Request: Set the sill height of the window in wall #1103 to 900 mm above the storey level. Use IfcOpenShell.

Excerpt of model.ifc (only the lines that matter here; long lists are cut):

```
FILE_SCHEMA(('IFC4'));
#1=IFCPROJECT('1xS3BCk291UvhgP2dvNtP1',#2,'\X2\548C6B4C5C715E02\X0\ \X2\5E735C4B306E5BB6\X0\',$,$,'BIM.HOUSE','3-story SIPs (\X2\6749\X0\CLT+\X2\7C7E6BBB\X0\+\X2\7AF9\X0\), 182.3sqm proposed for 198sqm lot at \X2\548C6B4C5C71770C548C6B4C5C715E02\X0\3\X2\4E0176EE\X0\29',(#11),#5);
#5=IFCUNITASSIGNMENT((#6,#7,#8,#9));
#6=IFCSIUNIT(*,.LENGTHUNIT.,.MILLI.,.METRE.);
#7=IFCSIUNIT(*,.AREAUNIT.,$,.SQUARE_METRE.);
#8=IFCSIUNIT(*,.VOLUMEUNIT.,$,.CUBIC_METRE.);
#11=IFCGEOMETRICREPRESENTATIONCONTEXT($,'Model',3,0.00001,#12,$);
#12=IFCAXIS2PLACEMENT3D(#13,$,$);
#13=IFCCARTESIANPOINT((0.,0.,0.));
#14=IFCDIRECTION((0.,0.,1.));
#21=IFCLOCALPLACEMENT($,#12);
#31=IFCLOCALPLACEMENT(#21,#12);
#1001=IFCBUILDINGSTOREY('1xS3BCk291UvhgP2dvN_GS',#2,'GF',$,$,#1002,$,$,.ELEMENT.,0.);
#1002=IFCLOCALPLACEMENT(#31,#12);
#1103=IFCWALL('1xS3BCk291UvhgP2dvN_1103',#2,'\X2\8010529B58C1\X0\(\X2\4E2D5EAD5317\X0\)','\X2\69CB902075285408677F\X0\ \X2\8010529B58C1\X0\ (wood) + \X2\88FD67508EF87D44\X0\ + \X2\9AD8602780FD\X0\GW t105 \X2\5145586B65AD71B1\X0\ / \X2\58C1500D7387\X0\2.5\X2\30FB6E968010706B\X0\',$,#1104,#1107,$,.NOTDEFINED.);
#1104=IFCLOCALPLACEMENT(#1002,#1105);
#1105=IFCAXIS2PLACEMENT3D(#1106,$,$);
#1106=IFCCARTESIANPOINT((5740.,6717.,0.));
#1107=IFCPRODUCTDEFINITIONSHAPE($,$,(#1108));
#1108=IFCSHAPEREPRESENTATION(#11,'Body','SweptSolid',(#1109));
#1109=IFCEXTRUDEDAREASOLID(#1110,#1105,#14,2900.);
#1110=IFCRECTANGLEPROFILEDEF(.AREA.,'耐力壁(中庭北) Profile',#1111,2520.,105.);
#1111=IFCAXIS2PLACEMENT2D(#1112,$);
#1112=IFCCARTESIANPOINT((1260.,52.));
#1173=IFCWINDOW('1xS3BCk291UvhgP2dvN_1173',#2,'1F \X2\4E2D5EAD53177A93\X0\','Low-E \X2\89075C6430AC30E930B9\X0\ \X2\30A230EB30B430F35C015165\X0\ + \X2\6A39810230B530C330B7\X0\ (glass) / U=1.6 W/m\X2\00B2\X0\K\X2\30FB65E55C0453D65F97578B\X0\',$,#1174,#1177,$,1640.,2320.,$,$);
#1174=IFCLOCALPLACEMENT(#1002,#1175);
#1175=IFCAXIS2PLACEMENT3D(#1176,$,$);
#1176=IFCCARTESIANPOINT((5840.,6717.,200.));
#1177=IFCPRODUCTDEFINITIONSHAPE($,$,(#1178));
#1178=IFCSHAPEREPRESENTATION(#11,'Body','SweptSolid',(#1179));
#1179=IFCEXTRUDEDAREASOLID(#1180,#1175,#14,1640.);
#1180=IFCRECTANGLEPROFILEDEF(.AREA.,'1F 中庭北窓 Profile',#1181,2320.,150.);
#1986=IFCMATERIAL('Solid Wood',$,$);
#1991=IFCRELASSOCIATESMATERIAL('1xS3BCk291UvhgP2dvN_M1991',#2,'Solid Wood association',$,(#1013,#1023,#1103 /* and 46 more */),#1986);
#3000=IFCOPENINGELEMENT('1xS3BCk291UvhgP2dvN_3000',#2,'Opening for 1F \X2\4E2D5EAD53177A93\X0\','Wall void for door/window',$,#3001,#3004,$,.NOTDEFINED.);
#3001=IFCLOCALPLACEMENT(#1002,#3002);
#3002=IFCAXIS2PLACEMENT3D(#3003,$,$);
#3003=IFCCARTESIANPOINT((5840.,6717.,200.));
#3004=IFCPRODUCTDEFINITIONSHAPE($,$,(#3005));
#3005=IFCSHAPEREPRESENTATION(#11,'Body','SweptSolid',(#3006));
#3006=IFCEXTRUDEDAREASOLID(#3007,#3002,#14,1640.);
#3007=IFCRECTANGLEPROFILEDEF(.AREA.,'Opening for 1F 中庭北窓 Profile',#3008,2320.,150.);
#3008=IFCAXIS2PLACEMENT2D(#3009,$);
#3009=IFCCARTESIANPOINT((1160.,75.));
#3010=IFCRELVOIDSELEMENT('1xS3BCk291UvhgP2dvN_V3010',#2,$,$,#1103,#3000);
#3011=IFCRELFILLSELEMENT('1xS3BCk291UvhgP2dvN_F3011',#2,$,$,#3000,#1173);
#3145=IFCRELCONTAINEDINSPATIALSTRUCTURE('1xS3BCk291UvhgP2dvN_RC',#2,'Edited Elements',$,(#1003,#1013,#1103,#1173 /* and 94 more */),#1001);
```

```python
import numpy as np
import ifcopenshell
import ifcopenshell.api.geometry
import ifcopenshell.geom
import ifcopenshell.util.element
import ifcopenshell.util.placement
import ifcopenshell.util.shape
import ifcopenshell.util.unit

model = ifcopenshell.open("model.ifc")
unit_scale = ifcopenshell.util.unit.calculate_unit_scale(model)

window = model.by_guid("1xS3BCk291UvhgP2dvN_1173")
opening = window.FillsVoids[0].RelatingOpeningElement
storey = ifcopenshell.util.element.get_container(window, ifc_class="IfcBuildingStorey")
level = ifcopenshell.util.placement.get_local_placement(storey.ObjectPlacement)[2, 3]

# The opening's origin need not be at the sill, so measure its lowest point.
shape = ifcopenshell.geom.create_shape(ifcopenshell.geom.settings(), opening)
bottom = ifcopenshell.util.shape.get_shape_bottom_elevation(shape, shape.geometry) / unit_scale
dz = level + 900.0 - bottom

shift = np.array([0.0, 0.0, dz])
# The window is not placed relative to its opening, so move both.
for product in (opening, window):
    matrix = ifcopenshell.util.placement.get_local_placement(product.ObjectPlacement)
    matrix[:3, 3] += shift
    ifcopenshell.api.geometry.edit_object_placement(model, product=product, matrix=matrix, is_si=False)

print(f"moved by {dz * unit_scale:+.3f} m")

model.write("model_v2.ifc")
```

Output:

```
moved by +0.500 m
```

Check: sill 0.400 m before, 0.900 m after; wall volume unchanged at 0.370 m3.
